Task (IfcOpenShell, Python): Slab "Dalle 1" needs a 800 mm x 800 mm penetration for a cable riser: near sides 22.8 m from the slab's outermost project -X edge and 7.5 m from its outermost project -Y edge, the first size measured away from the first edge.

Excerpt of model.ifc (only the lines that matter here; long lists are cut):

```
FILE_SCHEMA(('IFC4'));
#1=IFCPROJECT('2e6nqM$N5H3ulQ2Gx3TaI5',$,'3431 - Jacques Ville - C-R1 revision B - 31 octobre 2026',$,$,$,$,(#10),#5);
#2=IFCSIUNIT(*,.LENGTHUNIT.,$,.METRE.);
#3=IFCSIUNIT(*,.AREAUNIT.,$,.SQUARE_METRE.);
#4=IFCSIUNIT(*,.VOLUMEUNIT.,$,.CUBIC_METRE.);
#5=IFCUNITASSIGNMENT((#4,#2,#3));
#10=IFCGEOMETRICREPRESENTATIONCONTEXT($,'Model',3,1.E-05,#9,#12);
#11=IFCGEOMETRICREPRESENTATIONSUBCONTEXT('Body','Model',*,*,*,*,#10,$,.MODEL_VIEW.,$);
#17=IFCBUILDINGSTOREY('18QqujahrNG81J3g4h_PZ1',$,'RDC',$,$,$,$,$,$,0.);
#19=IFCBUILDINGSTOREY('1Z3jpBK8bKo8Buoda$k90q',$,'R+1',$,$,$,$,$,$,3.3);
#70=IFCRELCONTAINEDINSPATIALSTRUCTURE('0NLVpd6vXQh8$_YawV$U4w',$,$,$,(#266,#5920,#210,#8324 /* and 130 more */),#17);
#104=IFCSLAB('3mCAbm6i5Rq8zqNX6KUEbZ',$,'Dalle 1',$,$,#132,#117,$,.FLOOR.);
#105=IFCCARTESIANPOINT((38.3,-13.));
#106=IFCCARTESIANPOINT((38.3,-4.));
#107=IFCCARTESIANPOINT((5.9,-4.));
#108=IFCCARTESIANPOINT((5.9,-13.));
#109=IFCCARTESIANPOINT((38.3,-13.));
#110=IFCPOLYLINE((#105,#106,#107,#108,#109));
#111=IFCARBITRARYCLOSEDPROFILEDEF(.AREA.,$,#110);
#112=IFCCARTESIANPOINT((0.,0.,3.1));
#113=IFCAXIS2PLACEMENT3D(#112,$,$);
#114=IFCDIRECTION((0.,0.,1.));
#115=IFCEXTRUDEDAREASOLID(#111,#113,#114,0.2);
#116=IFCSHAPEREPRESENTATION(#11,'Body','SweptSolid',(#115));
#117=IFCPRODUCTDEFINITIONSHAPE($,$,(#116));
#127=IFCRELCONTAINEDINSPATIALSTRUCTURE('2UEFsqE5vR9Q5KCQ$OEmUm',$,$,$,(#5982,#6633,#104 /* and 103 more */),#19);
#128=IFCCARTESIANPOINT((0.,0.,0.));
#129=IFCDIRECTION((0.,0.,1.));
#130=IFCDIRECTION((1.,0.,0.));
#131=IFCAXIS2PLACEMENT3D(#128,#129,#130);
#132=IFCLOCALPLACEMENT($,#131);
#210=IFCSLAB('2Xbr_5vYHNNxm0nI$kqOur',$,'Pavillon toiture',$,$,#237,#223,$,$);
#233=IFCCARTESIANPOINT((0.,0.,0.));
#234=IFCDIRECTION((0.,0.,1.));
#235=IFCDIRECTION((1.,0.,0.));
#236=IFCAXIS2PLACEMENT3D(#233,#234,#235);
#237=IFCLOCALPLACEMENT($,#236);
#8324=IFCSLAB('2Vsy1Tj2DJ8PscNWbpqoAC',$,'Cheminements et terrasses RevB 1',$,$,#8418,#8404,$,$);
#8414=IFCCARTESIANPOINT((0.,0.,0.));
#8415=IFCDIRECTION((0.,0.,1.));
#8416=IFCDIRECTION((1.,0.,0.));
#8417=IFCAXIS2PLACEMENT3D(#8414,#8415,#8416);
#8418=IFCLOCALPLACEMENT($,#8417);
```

```python
import numpy as np
import ifcopenshell
import ifcopenshell.api.feature
import ifcopenshell.api.geometry
import ifcopenshell.api.root
import ifcopenshell.geom
import ifcopenshell.util.placement
import ifcopenshell.util.representation
import ifcopenshell.util.shape
import ifcopenshell.util.unit

model = ifcopenshell.open("model.ifc")
unit_scale = ifcopenshell.util.unit.calculate_unit_scale(model)
settings = ifcopenshell.geom.settings()


def volume(element):
    """Net volume in cubic metres, openings subtracted."""
    shape = ifcopenshell.geom.create_shape(settings, element)
    return ifcopenshell.util.shape.get_volume(shape.geometry)


slab = model.by_id(104)
before = volume(slab)

# Extent in the slab's own axes, in metres. The edges named are its -X and -Y sides.
slab_shape = ifcopenshell.geom.create_shape(settings, slab)
vertices = ifcopenshell.util.shape.get_vertices(slab_shape.geometry)
x_min, y_min, bottom = vertices.min(axis=0)
top = vertices[:, 2].max()

opening = ifcopenshell.api.root.create_entity(model, ifc_class="IfcOpeningElement", name="Cable riser opening", predefined_type="OPENING")
context = ifcopenshell.util.representation.get_context(model, "Model", "Body", "MODEL_VIEW")
width, depth = 0.8, 0.8
outline = [(0.0, 0.0), (width, 0.0), (width, depth), (0.0, depth), (0.0, 0.0)]
# Overshoot both faces by 50 mm so the cut is clean.
shape = ifcopenshell.api.geometry.add_slab_representation(
    model, context=context, depth=top - bottom + 0.1, polyline=outline
)
ifcopenshell.api.geometry.assign_representation(model, product=opening, representation=shape)

matrix = ifcopenshell.util.placement.get_local_placement(slab.ObjectPlacement)
matrix[:, 3] = matrix @ np.append(np.array([x_min + 22.8, y_min + 7.5, bottom - 0.05]) / unit_scale, 1.0)
ifcopenshell.api.geometry.edit_object_placement(model, product=opening, matrix=matrix, is_si=False)
ifcopenshell.api.feature.add_feature(model, feature=opening, element=slab)

after = volume(slab)

print(f"slab volume {before:.3f} -> {after:.3f} m3")

model.write("model-out.ifc")
```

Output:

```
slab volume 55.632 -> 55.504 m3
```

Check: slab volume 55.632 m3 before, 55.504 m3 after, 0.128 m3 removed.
